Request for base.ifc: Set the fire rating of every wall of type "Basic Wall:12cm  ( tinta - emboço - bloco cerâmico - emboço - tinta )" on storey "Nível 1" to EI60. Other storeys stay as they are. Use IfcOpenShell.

First a look at what the model holds.

```python
import ifcopenshell
import ifcopenshell.util.element

model = ifcopenshell.open("base.ifc")
print(model.schema)
storey = next(s for s in model.by_type("IfcBuildingStorey") if s.Name == "Nível 1")
walls = [e for e in ifcopenshell.util.element.get_decomposition(storey) if e.is_a("IfcWall")]
seen = {}
for e in walls:
    element_type = ifcopenshell.util.element.get_type(e)
    key = (element_type.Name if element_type != e and element_type else None, ifcopenshell.util.element.get_pset(e, "Pset_WallCommon", "FireRating"))
    seen[key] = seen.get(key, 0) + 1
for (name, value), count in sorted(seen.items(), key=str):
    print(count, "x", name, "|", value)
```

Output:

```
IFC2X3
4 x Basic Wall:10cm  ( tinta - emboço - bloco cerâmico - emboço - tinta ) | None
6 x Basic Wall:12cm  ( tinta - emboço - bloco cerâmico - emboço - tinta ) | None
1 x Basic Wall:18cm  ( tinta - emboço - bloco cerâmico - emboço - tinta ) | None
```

```python
import ifcopenshell
import ifcopenshell.api.pset
import ifcopenshell.util.element

model = ifcopenshell.open("base.ifc")

storey = next(s for s in model.by_type("IfcBuildingStorey") if s.Name == "Nível 1")
walls = [e for e in ifcopenshell.util.element.get_decomposition(storey) if e.is_a("IfcWall")]

count = 0
for e in walls:
    element_type = ifcopenshell.util.element.get_type(e)
    if element_type in (None, e) or element_type.Name != "Basic Wall:12cm  ( tinta - emboço - bloco cerâmico - emboço - tinta )":
        continue
    # add_pset returns the element's existing set when there is one.
    pset = ifcopenshell.api.pset.add_pset(model, product=e, name="Pset_WallCommon")
    ifcopenshell.api.pset.edit_pset(model, pset=pset, properties={"FireRating": "EI60"})
    count += 1

print(count, "walls updated")

model.write("base_updated.ifc")
```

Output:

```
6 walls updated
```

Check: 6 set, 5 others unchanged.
